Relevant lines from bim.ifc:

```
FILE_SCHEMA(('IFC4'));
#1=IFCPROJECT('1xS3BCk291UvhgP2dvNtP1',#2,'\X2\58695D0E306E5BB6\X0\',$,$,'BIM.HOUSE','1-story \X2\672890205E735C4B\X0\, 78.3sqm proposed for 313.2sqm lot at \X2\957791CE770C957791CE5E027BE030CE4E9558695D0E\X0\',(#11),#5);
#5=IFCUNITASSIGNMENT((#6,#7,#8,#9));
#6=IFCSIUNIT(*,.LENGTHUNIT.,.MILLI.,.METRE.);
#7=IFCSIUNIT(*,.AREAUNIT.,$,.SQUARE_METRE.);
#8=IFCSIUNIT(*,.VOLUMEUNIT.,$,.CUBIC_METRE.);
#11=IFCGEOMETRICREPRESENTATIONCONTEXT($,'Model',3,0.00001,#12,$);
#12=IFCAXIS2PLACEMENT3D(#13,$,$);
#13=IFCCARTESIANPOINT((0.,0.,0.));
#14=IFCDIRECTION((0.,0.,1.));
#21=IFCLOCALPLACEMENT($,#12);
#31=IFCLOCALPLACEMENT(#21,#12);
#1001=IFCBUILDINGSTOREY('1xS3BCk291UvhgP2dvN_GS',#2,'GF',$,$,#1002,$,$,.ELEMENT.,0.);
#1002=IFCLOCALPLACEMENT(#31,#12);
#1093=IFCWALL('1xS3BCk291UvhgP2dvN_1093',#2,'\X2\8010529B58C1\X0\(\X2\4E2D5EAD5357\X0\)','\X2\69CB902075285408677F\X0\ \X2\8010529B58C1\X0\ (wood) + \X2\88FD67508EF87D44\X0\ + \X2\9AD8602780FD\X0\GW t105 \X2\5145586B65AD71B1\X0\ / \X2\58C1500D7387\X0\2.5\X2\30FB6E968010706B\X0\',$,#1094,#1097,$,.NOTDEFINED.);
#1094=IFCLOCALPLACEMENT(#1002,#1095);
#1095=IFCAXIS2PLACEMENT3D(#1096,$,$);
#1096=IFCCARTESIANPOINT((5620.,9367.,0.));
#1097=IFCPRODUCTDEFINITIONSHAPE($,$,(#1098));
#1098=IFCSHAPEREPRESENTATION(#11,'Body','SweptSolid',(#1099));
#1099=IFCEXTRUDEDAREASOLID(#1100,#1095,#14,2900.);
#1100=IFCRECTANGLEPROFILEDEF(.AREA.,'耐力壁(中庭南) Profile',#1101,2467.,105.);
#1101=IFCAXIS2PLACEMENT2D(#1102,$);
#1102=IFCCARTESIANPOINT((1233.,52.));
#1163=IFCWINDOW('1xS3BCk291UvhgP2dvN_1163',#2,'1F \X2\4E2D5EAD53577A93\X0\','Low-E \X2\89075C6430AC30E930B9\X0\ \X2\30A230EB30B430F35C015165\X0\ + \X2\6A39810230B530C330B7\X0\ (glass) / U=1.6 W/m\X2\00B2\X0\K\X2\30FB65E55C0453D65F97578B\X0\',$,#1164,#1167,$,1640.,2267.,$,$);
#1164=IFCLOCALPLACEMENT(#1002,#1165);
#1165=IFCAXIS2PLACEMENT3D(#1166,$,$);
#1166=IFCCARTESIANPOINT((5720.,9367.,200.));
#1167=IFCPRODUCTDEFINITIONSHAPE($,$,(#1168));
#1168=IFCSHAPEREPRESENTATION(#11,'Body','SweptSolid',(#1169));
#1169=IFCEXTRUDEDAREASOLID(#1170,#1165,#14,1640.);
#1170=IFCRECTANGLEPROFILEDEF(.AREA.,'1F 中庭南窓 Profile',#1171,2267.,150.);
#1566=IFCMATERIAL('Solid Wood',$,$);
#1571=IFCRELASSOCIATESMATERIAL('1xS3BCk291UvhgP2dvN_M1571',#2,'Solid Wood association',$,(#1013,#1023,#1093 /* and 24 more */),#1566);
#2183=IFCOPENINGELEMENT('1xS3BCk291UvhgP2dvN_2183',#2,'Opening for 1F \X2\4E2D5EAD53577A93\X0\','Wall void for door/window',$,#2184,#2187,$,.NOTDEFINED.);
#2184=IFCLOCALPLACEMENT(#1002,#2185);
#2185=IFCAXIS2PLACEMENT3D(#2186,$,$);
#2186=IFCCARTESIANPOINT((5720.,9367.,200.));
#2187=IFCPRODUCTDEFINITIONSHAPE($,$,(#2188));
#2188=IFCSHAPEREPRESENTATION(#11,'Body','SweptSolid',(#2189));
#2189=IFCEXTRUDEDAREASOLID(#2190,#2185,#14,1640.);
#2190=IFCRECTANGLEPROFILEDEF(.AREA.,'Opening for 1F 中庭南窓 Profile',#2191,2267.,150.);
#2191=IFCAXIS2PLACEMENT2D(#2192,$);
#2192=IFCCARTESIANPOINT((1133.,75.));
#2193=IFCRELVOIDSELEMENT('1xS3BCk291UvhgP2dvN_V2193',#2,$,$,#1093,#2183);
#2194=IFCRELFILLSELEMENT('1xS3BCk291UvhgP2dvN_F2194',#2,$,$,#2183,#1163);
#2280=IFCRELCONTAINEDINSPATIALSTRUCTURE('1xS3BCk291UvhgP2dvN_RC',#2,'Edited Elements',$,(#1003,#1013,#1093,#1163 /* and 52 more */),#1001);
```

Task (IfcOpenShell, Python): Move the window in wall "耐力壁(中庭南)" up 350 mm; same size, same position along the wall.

```python
import numpy as np
import ifcopenshell
import ifcopenshell.api.geometry
import ifcopenshell.util.placement
import ifcopenshell.util.unit

model = ifcopenshell.open("bim.ifc")
unit_scale = ifcopenshell.util.unit.calculate_unit_scale(model)

window = model.by_guid("1xS3BCk291UvhgP2dvN_1163")
opening = window.FillsVoids[0].RelatingOpeningElement
dz = 350.0

shift = np.array([0.0, 0.0, dz])
# The window is not placed relative to its opening, so move both.
for product in (opening, window):
    matrix = ifcopenshell.util.placement.get_local_placement(product.ObjectPlacement)
    matrix[:3, 3] += shift
    ifcopenshell.api.geometry.edit_object_placement(model, product=product, matrix=matrix, is_si=False)

print(f"moved by {dz * unit_scale:+.3f} m")

model.write("bim-out.ifc")
```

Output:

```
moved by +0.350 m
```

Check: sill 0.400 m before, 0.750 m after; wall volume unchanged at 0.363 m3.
